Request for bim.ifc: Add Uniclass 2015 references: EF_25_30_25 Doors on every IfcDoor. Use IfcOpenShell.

First a look at what the model holds.

```python
import ifcopenshell

model = ifcopenshell.open("bim.ifc")
print(model.schema)
print("classifications:", [c.Name for c in model.by_type("IfcClassification")])
for ifc_class in ("IfcDoor", "IfcRoof", "IfcStair", "IfcWall", "IfcWindow"):
    print(ifc_class, len(model.by_type(ifc_class)))
```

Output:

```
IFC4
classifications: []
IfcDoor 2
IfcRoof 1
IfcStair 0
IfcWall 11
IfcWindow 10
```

```python
import ifcopenshell
import ifcopenshell.api.classification

model = ifcopenshell.open("bim.ifc")

system = ifcopenshell.api.classification.add_classification(model, classification="Uniclass 2015")

codes = {
    "IfcDoor": ("EF_25_30_25", "Doors"),
}
for ifc_class, (code, name) in codes.items():
    products = model.by_type(ifc_class)
    ifcopenshell.api.classification.add_reference(
        model, products=products, classification=system, identification=code, name=name
    )
    print(code, len(products))

model.write("bim_rev.ifc")
```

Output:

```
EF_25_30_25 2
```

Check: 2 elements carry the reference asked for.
